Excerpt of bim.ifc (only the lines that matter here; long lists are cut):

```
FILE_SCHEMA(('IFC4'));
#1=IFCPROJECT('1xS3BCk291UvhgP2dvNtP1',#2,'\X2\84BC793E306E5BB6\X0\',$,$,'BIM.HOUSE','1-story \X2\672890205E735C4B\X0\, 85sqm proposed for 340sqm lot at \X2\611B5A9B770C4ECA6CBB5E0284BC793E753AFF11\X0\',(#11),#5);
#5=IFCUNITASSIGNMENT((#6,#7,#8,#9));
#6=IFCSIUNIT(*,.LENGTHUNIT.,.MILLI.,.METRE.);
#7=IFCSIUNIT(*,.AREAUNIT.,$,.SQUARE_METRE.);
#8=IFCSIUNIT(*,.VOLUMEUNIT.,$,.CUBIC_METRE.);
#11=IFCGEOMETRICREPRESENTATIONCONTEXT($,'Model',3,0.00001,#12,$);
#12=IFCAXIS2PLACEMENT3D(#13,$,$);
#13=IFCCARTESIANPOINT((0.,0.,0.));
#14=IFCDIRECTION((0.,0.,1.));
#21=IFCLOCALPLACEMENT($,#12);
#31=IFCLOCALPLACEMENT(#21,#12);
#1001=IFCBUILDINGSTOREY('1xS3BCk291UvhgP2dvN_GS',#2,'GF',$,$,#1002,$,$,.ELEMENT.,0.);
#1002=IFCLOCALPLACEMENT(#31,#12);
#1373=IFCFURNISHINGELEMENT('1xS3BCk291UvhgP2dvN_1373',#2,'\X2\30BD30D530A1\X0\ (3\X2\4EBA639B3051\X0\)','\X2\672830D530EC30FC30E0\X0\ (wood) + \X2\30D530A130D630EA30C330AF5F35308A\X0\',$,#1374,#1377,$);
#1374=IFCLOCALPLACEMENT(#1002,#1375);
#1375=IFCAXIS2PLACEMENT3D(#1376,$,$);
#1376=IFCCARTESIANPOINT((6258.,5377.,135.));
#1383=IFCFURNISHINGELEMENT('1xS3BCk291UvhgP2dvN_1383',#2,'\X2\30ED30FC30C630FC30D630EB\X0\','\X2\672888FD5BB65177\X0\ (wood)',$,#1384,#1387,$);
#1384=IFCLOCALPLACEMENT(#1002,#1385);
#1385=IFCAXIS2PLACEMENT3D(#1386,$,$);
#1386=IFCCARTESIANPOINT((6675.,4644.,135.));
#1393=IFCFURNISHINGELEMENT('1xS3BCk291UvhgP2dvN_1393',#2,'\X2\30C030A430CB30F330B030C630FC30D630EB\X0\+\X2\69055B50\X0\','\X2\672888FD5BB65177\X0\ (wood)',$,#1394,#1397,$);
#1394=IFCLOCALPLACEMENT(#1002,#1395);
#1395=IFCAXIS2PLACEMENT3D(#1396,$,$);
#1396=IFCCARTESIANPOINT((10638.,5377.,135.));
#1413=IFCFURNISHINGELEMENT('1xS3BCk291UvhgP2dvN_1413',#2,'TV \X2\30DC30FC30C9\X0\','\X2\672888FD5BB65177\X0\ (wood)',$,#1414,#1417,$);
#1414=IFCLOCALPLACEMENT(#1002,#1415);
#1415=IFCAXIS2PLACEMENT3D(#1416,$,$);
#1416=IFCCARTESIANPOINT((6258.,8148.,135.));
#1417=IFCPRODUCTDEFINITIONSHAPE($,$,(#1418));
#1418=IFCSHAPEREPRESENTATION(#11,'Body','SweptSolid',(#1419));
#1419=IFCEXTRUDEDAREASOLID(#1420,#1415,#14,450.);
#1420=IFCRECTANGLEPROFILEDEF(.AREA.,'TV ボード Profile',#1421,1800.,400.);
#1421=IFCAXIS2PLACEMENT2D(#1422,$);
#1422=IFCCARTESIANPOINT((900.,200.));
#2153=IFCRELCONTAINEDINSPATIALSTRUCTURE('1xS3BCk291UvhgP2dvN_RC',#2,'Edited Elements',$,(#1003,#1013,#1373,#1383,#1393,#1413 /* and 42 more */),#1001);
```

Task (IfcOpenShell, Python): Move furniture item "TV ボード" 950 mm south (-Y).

```python
import ifcopenshell
import ifcopenshell.api.geometry
import ifcopenshell.util.placement
import ifcopenshell.util.unit

model = ifcopenshell.open("bim.ifc")
unit_scale = ifcopenshell.util.unit.calculate_unit_scale(model)

item = model.by_id(1413)
matrix = ifcopenshell.util.placement.get_local_placement(item.ObjectPlacement)
matrix[1, 3] -= 0.95 / unit_scale
ifcopenshell.api.geometry.edit_object_placement(model, product=item, matrix=matrix, is_si=False)

print(ifcopenshell.util.placement.get_local_placement(item.ObjectPlacement).round(3) + 0.0)

model.write("bim_rev.ifc")
```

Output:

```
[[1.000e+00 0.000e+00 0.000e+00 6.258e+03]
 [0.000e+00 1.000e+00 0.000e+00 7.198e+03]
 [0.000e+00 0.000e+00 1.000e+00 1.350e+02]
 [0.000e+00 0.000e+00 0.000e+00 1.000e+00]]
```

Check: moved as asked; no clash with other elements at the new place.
